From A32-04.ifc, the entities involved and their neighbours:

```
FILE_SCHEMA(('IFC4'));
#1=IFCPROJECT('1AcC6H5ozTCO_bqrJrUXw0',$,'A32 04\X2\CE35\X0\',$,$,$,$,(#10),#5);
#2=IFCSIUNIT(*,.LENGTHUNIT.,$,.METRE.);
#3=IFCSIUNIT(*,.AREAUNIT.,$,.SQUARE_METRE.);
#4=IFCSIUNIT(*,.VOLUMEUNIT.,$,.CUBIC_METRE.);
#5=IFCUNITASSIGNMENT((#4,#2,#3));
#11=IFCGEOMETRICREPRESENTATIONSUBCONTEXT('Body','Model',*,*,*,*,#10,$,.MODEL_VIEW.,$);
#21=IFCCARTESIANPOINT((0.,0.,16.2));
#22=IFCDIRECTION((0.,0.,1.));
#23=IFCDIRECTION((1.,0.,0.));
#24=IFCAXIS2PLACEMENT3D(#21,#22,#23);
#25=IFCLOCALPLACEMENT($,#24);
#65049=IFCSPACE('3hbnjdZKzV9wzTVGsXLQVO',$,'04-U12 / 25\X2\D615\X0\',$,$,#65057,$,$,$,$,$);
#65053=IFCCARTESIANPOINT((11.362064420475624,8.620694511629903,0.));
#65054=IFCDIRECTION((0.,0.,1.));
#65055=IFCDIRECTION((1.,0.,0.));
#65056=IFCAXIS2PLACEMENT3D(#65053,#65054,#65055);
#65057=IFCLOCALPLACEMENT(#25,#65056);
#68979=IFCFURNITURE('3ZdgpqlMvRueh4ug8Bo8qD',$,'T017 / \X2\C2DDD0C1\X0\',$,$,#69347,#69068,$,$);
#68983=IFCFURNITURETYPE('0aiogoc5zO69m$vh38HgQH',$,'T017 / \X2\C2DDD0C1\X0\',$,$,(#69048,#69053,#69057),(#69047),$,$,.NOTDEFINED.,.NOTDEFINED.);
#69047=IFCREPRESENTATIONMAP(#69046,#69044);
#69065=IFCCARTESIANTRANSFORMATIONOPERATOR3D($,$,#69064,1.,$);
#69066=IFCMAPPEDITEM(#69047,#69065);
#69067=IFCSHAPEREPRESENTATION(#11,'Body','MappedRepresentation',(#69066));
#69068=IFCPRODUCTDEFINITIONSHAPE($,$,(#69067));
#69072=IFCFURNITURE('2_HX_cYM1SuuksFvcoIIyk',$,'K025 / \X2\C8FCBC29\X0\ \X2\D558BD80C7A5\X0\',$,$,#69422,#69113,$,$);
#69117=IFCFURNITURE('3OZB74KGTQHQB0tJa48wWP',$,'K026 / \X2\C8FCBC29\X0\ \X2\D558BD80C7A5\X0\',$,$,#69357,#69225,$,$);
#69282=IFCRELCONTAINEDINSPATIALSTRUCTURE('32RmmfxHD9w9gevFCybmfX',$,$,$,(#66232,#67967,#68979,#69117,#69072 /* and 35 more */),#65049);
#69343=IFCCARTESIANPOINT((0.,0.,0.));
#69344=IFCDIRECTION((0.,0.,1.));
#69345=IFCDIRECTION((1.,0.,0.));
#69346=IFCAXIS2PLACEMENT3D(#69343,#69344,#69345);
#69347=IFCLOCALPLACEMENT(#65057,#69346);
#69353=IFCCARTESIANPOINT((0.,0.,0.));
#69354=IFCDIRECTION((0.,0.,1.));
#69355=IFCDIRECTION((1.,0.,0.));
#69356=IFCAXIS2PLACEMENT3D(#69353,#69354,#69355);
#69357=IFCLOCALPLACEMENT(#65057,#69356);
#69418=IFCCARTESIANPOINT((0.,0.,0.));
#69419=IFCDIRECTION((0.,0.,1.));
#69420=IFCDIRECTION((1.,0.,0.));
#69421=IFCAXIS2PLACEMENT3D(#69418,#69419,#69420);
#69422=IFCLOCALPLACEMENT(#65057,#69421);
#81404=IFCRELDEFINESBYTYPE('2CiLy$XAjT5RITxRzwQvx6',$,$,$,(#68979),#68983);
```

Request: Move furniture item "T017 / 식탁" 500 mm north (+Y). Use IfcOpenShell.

```python
import ifcopenshell
import ifcopenshell.api.geometry
import ifcopenshell.util.placement

model = ifcopenshell.open("A32-04.ifc")

item = model.by_guid("3ZdgpqlMvRueh4ug8Bo8qD")
matrix = ifcopenshell.util.placement.get_local_placement(item.ObjectPlacement)
matrix[1, 3] += 0.5
ifcopenshell.api.geometry.edit_object_placement(model, product=item, matrix=matrix, is_si=False)

print(ifcopenshell.util.placement.get_local_placement(item.ObjectPlacement).round(3) + 0.0)

model.write("A32-04_rev.ifc")
```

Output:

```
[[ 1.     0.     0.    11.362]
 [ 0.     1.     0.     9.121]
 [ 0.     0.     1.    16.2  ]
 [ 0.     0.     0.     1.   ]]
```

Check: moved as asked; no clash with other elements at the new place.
